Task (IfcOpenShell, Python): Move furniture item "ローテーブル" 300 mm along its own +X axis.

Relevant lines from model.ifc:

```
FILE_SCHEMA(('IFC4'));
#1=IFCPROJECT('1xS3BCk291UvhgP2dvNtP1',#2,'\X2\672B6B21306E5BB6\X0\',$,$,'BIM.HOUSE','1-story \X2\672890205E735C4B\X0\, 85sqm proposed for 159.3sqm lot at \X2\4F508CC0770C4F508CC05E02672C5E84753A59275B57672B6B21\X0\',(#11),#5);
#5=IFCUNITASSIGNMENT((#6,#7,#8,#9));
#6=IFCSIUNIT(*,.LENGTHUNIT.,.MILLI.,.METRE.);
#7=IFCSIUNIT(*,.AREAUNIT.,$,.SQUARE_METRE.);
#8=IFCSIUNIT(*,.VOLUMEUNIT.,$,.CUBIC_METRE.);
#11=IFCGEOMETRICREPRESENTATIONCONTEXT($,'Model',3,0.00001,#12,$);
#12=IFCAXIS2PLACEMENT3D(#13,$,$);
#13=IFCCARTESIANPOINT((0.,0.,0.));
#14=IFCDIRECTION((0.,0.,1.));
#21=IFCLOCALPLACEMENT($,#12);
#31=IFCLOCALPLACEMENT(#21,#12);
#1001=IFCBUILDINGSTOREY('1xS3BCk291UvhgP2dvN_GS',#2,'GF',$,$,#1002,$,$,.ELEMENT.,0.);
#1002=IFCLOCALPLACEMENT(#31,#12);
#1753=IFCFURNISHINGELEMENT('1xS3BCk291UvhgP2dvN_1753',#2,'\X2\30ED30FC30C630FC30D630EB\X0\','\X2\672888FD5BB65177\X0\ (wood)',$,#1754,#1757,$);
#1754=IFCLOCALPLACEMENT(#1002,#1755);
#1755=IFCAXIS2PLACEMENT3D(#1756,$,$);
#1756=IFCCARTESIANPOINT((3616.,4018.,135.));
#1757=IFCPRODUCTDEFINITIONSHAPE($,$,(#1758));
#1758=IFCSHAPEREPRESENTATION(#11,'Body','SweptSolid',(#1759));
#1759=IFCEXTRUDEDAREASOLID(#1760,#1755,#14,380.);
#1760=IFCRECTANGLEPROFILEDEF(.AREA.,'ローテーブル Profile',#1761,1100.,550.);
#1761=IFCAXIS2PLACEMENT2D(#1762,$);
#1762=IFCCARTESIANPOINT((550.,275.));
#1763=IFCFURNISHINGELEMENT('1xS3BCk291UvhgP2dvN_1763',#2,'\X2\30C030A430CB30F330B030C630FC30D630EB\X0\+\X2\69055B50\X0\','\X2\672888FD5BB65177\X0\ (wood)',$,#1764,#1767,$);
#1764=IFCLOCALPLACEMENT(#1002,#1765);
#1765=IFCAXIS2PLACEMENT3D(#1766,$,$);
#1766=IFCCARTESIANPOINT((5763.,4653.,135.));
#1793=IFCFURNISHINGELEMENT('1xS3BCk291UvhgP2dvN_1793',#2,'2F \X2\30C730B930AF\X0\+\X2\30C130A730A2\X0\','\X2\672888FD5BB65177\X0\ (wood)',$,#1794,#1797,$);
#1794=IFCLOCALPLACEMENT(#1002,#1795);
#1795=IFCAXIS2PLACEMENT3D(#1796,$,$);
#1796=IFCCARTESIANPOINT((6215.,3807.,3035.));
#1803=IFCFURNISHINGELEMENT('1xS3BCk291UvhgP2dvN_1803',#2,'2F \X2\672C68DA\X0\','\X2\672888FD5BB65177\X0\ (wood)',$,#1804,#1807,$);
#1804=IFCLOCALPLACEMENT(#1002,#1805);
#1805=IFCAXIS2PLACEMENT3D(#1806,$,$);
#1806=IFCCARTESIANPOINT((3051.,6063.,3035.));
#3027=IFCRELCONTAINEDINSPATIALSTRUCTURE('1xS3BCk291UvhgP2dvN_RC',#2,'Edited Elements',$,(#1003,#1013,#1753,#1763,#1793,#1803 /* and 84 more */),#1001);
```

```python
import ifcopenshell
import ifcopenshell.api.geometry
import ifcopenshell.util.placement
import ifcopenshell.util.unit

model = ifcopenshell.open("model.ifc")
unit_scale = ifcopenshell.util.unit.calculate_unit_scale(model)

item = model.by_guid("1xS3BCk291UvhgP2dvN_1753")
matrix = ifcopenshell.util.placement.get_local_placement(item.ObjectPlacement)
matrix[:3, 3] += matrix[:3, 0] * 0.3 / unit_scale
ifcopenshell.api.geometry.edit_object_placement(model, product=item, matrix=matrix, is_si=False)

print(ifcopenshell.util.placement.get_local_placement(item.ObjectPlacement).round(3) + 0.0)

model.write("model_rev.ifc")
```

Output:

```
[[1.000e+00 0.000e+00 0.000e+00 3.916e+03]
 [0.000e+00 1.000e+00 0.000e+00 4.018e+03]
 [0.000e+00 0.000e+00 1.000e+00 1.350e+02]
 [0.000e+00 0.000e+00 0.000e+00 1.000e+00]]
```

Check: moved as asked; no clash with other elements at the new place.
